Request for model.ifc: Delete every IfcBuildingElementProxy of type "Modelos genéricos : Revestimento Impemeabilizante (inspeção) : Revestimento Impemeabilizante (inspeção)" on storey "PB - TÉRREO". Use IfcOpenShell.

First a look at what the model holds.

```python
import ifcopenshell
import ifcopenshell.util.element

model = ifcopenshell.open("model.ifc")
print(model.schema)
storey = next(s for s in model.by_type("IfcBuildingStorey") if s.Name == "PB - TÉRREO")
proxies = [e for e in ifcopenshell.util.element.get_decomposition(storey) if e.is_a("IfcBuildingElementProxy")]
seen = {}
for e in proxies:
    element_type = ifcopenshell.util.element.get_type(e)
    name = element_type.Name if element_type not in (None, e) else None
    seen[name] = seen.get(name, 0) + 1
for name, count in sorted(seen.items(), key=str):
    print(count, "x", name)
```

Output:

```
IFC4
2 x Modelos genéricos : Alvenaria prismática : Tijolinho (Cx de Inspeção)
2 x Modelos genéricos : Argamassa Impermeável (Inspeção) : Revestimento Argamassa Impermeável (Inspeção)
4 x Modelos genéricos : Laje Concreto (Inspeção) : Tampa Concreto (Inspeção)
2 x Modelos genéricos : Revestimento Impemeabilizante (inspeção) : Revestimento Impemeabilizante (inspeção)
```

```python
import ifcopenshell
import ifcopenshell.api.root
import ifcopenshell.util.element

model = ifcopenshell.open("model.ifc")

storey = next(s for s in model.by_type("IfcBuildingStorey") if s.Name == "PB - TÉRREO")
proxies = [e for e in ifcopenshell.util.element.get_decomposition(storey) if e.is_a("IfcBuildingElementProxy")]
targets = [e for e in proxies if (t := ifcopenshell.util.element.get_type(e)) not in (None, e) and t.Name == "Modelos genéricos : Revestimento Impemeabilizante (inspeção) : Revestimento Impemeabilizante (inspeção)"]

for e in targets:
    ifcopenshell.api.root.remove_product(model, product=e)
print(len(targets), "removed")

model.write("model_rev.ifc")
```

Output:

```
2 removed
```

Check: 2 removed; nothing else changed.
